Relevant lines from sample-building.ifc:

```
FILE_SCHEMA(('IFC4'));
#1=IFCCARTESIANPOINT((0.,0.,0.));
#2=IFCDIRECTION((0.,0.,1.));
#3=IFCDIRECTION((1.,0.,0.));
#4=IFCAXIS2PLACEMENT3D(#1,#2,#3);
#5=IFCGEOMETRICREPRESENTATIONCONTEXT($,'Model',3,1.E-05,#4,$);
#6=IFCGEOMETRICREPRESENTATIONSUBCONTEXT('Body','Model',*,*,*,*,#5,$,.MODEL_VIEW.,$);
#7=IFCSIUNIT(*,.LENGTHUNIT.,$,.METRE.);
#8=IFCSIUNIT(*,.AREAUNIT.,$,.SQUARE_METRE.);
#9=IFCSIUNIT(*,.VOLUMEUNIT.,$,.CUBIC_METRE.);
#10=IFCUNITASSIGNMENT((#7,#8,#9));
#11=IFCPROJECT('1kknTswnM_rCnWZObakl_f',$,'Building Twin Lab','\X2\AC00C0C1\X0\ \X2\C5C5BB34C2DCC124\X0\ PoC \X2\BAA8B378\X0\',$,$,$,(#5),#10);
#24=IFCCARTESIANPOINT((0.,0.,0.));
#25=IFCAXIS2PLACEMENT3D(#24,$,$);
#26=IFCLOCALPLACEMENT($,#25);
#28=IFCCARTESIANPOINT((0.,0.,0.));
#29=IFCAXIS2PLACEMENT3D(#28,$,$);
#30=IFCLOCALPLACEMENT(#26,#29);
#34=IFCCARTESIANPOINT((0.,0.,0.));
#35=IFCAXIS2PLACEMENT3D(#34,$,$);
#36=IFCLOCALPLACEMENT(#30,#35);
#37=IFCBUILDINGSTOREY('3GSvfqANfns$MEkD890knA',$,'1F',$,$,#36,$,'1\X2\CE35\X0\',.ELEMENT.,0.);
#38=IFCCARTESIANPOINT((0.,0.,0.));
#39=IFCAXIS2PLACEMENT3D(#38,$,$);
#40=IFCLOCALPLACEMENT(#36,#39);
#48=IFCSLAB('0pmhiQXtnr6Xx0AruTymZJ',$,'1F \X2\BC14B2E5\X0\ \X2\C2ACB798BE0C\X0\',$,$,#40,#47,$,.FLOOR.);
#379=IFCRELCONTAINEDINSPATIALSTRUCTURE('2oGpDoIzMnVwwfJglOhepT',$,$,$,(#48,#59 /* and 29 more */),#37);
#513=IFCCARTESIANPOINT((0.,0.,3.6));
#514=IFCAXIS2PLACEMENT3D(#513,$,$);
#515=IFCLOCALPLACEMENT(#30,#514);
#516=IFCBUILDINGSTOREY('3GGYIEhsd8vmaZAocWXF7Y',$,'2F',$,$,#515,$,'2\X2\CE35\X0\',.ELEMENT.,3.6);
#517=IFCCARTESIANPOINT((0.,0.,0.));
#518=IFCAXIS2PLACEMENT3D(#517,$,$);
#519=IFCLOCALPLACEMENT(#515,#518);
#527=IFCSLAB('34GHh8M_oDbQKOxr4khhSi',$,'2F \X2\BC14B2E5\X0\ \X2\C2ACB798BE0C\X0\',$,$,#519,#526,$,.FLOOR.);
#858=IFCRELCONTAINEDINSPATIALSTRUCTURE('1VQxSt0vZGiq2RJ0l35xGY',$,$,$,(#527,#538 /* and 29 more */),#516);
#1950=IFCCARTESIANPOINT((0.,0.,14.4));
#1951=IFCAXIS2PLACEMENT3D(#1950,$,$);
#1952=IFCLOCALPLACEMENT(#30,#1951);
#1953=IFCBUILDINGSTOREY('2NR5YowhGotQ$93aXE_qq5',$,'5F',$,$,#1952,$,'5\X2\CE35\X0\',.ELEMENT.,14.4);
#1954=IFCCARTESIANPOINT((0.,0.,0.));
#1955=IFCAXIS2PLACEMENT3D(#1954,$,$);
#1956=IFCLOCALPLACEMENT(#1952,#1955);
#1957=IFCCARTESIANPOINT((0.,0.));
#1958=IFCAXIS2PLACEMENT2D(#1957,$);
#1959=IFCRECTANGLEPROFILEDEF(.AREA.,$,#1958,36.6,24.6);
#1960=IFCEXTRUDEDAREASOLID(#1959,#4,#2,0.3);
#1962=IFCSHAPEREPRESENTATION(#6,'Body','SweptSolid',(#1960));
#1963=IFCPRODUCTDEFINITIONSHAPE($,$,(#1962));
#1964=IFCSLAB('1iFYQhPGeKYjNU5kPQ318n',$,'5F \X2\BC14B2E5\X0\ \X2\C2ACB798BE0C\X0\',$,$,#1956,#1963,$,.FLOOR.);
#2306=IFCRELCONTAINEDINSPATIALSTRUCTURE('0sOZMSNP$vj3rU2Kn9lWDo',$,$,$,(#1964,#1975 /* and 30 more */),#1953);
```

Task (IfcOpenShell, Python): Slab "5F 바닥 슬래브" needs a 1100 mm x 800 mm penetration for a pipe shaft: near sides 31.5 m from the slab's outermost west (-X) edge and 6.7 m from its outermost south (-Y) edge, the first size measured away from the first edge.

```python
import numpy as np
import ifcopenshell
import ifcopenshell.api.feature
import ifcopenshell.api.geometry
import ifcopenshell.api.root
import ifcopenshell.geom
import ifcopenshell.util.placement
import ifcopenshell.util.representation
import ifcopenshell.util.shape
import ifcopenshell.util.unit

model = ifcopenshell.open("sample-building.ifc")
unit_scale = ifcopenshell.util.unit.calculate_unit_scale(model)
settings = ifcopenshell.geom.settings()


def volume(element):
    """Net volume in cubic metres, openings subtracted."""
    shape = ifcopenshell.geom.create_shape(settings, element)
    return ifcopenshell.util.shape.get_volume(shape.geometry)


slab = model.by_guid("1iFYQhPGeKYjNU5kPQ318n")
before = volume(slab)

# Extent in the slab's own axes, in metres. The edges named are its -X and -Y sides.
slab_shape = ifcopenshell.geom.create_shape(settings, slab)
vertices = ifcopenshell.util.shape.get_vertices(slab_shape.geometry)
x_min, y_min, bottom = vertices.min(axis=0)
top = vertices[:, 2].max()

opening = ifcopenshell.api.root.create_entity(model, ifc_class="IfcOpeningElement", name="Pipe shaft opening", predefined_type="OPENING")
context = ifcopenshell.util.representation.get_context(model, "Model", "Body", "MODEL_VIEW")
width, depth = 1.1, 0.8
outline = [(0.0, 0.0), (width, 0.0), (width, depth), (0.0, depth), (0.0, 0.0)]
# Overshoot both faces by 50 mm so the cut is clean.
shape = ifcopenshell.api.geometry.add_slab_representation(
    model, context=context, depth=top - bottom + 0.1, polyline=outline
)
ifcopenshell.api.geometry.assign_representation(model, product=opening, representation=shape)

matrix = ifcopenshell.util.placement.get_local_placement(slab.ObjectPlacement)
matrix[:, 3] = matrix @ np.append(np.array([x_min + 31.5, y_min + 6.7, bottom - 0.05]) / unit_scale, 1.0)
ifcopenshell.api.geometry.edit_object_placement(model, product=opening, matrix=matrix, is_si=False)
ifcopenshell.api.feature.add_feature(model, feature=opening, element=slab)

after = volume(slab)

print(f"slab volume {before:.3f} -> {after:.3f} m3")

model.write("sample-building_v2.ifc")
```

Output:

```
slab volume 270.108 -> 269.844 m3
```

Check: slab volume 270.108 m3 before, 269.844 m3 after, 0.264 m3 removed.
